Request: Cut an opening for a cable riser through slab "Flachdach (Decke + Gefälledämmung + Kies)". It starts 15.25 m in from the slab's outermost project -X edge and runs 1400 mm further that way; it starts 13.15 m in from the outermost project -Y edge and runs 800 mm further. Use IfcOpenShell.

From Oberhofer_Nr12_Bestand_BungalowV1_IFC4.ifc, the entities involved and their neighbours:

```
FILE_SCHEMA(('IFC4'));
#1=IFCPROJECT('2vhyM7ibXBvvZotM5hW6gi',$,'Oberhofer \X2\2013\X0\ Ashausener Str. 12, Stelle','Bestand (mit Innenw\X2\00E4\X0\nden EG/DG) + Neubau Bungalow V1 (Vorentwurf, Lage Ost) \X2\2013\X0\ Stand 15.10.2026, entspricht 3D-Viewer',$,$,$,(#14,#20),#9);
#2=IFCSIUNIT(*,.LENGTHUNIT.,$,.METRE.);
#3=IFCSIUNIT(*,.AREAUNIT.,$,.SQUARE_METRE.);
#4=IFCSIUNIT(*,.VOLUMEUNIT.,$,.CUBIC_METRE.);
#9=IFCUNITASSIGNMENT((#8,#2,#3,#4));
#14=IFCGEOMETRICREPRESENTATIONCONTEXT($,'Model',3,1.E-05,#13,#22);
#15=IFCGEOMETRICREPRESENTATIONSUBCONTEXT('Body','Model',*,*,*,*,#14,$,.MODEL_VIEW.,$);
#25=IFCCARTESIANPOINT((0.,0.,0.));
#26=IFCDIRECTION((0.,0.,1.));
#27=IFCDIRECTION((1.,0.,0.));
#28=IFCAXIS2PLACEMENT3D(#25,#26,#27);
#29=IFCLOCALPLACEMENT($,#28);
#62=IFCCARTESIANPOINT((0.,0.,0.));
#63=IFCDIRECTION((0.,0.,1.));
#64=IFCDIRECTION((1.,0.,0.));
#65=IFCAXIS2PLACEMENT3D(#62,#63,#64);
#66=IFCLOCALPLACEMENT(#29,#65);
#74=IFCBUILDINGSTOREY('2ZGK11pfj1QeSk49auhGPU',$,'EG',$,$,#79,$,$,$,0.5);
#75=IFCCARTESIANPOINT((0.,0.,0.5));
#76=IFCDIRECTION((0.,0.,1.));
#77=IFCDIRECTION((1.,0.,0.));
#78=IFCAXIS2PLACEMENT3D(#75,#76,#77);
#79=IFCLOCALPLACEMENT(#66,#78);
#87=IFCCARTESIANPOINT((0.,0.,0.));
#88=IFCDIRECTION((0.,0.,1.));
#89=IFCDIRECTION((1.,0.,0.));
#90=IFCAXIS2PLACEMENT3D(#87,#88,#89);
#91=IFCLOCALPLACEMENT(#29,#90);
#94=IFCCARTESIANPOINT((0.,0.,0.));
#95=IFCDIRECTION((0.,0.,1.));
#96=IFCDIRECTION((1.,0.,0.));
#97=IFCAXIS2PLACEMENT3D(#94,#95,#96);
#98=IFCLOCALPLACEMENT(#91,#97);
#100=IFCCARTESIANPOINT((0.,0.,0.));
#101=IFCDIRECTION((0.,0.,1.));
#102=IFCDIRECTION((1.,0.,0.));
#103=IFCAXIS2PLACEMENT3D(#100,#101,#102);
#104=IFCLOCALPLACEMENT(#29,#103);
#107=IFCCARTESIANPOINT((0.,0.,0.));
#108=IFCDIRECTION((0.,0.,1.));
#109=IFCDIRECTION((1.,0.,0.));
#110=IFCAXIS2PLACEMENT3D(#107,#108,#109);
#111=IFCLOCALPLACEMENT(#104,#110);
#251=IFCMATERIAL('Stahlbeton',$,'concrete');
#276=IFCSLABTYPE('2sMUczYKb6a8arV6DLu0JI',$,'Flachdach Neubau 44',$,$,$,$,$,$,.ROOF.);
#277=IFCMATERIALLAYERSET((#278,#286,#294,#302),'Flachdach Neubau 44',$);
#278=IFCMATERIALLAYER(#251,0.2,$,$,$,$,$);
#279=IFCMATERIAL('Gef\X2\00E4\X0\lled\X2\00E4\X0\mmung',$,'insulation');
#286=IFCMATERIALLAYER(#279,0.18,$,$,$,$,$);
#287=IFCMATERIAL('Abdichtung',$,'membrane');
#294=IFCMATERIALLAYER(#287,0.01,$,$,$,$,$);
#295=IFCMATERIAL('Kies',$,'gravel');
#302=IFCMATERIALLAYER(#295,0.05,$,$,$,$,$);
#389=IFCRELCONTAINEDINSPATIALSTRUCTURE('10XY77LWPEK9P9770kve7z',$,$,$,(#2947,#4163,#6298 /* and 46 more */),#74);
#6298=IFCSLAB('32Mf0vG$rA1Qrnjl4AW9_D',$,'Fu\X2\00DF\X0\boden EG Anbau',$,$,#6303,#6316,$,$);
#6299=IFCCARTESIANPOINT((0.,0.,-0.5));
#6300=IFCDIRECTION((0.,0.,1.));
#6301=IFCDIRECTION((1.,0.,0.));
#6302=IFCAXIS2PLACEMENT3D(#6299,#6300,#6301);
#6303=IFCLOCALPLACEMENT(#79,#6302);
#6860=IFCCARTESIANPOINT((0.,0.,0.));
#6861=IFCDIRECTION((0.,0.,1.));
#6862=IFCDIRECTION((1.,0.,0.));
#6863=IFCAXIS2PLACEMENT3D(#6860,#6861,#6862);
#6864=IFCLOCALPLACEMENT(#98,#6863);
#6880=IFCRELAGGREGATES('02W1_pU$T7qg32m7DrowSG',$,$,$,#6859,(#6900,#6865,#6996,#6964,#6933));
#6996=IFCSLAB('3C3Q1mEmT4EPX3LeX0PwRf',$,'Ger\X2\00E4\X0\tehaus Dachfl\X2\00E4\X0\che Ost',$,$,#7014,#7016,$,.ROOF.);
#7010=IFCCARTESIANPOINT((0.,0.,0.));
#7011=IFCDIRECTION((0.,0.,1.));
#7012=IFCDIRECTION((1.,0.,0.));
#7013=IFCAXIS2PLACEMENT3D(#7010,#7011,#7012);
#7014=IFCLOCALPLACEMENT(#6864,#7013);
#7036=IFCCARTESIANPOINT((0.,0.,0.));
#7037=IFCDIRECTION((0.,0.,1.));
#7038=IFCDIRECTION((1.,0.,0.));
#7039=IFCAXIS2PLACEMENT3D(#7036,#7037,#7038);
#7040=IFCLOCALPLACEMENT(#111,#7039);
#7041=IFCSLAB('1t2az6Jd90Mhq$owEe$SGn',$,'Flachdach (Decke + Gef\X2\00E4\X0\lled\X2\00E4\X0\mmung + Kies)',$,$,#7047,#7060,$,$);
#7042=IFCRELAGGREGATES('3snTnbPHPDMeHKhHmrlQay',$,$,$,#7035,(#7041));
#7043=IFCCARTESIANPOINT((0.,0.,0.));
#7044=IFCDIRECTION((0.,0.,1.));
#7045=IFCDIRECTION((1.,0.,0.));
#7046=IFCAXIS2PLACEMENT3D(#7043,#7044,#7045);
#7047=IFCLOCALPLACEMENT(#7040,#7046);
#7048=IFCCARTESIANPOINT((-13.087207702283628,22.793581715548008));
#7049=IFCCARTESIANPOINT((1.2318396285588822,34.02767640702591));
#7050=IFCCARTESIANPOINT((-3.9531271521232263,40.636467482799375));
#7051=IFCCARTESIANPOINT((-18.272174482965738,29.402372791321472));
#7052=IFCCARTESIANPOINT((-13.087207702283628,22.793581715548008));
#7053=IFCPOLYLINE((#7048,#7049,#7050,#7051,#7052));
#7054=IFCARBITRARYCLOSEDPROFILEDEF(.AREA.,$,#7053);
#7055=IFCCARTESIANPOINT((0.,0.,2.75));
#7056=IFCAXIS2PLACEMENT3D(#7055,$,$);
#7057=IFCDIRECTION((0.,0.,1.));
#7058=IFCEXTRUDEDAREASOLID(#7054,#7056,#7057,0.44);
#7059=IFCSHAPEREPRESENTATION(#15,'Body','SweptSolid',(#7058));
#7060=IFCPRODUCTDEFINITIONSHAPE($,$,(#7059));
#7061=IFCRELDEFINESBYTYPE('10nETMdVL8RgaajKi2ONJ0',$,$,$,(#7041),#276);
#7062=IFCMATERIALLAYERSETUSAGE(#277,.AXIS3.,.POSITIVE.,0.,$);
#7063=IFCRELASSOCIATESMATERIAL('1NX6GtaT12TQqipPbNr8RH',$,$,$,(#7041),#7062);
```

```python
import numpy as np
import ifcopenshell
import ifcopenshell.api.feature
import ifcopenshell.api.geometry
import ifcopenshell.api.root
import ifcopenshell.geom
import ifcopenshell.util.placement
import ifcopenshell.util.representation
import ifcopenshell.util.shape
import ifcopenshell.util.unit

model = ifcopenshell.open("Oberhofer_Nr12_Bestand_BungalowV1_IFC4.ifc")
unit_scale = ifcopenshell.util.unit.calculate_unit_scale(model)
settings = ifcopenshell.geom.settings()


def volume(element):
    """Net volume in cubic metres, openings subtracted."""
    shape = ifcopenshell.geom.create_shape(settings, element)
    return ifcopenshell.util.shape.get_volume(shape.geometry)


slab = model.by_guid("1t2az6Jd90Mhq$owEe$SGn")
before = volume(slab)

# Extent in the slab's own axes, in metres. The edges named are its -X and -Y sides.
slab_shape = ifcopenshell.geom.create_shape(settings, slab)
vertices = ifcopenshell.util.shape.get_vertices(slab_shape.geometry)
x_min, y_min, bottom = vertices.min(axis=0)
top = vertices[:, 2].max()

opening = ifcopenshell.api.root.create_entity(model, ifc_class="IfcOpeningElement", name="Cable riser opening", predefined_type="OPENING")
context = ifcopenshell.util.representation.get_context(model, "Model", "Body", "MODEL_VIEW")
width, depth = 1.4, 0.8
outline = [(0.0, 0.0), (width, 0.0), (width, depth), (0.0, depth), (0.0, 0.0)]
# Overshoot both faces by 50 mm so the cut is clean.
shape = ifcopenshell.api.geometry.add_slab_representation(
    model, context=context, depth=top - bottom + 0.1, polyline=outline
)
ifcopenshell.api.geometry.assign_representation(model, product=opening, representation=shape)

matrix = ifcopenshell.util.placement.get_local_placement(slab.ObjectPlacement)
matrix[:, 3] = matrix @ np.append(np.array([x_min + 15.25, y_min + 13.15, bottom - 0.05]) / unit_scale, 1.0)
ifcopenshell.api.geometry.edit_object_placement(model, product=opening, matrix=matrix, is_si=False)
ifcopenshell.api.feature.add_feature(model, feature=opening, element=slab)

after = volume(slab)

print(f"slab volume {before:.3f} -> {after:.3f} m3")

model.write("Oberhofer_Nr12_Bestand_BungalowV1_IFC4_edited.ifc")
```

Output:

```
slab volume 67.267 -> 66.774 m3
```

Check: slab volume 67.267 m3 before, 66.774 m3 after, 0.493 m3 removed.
